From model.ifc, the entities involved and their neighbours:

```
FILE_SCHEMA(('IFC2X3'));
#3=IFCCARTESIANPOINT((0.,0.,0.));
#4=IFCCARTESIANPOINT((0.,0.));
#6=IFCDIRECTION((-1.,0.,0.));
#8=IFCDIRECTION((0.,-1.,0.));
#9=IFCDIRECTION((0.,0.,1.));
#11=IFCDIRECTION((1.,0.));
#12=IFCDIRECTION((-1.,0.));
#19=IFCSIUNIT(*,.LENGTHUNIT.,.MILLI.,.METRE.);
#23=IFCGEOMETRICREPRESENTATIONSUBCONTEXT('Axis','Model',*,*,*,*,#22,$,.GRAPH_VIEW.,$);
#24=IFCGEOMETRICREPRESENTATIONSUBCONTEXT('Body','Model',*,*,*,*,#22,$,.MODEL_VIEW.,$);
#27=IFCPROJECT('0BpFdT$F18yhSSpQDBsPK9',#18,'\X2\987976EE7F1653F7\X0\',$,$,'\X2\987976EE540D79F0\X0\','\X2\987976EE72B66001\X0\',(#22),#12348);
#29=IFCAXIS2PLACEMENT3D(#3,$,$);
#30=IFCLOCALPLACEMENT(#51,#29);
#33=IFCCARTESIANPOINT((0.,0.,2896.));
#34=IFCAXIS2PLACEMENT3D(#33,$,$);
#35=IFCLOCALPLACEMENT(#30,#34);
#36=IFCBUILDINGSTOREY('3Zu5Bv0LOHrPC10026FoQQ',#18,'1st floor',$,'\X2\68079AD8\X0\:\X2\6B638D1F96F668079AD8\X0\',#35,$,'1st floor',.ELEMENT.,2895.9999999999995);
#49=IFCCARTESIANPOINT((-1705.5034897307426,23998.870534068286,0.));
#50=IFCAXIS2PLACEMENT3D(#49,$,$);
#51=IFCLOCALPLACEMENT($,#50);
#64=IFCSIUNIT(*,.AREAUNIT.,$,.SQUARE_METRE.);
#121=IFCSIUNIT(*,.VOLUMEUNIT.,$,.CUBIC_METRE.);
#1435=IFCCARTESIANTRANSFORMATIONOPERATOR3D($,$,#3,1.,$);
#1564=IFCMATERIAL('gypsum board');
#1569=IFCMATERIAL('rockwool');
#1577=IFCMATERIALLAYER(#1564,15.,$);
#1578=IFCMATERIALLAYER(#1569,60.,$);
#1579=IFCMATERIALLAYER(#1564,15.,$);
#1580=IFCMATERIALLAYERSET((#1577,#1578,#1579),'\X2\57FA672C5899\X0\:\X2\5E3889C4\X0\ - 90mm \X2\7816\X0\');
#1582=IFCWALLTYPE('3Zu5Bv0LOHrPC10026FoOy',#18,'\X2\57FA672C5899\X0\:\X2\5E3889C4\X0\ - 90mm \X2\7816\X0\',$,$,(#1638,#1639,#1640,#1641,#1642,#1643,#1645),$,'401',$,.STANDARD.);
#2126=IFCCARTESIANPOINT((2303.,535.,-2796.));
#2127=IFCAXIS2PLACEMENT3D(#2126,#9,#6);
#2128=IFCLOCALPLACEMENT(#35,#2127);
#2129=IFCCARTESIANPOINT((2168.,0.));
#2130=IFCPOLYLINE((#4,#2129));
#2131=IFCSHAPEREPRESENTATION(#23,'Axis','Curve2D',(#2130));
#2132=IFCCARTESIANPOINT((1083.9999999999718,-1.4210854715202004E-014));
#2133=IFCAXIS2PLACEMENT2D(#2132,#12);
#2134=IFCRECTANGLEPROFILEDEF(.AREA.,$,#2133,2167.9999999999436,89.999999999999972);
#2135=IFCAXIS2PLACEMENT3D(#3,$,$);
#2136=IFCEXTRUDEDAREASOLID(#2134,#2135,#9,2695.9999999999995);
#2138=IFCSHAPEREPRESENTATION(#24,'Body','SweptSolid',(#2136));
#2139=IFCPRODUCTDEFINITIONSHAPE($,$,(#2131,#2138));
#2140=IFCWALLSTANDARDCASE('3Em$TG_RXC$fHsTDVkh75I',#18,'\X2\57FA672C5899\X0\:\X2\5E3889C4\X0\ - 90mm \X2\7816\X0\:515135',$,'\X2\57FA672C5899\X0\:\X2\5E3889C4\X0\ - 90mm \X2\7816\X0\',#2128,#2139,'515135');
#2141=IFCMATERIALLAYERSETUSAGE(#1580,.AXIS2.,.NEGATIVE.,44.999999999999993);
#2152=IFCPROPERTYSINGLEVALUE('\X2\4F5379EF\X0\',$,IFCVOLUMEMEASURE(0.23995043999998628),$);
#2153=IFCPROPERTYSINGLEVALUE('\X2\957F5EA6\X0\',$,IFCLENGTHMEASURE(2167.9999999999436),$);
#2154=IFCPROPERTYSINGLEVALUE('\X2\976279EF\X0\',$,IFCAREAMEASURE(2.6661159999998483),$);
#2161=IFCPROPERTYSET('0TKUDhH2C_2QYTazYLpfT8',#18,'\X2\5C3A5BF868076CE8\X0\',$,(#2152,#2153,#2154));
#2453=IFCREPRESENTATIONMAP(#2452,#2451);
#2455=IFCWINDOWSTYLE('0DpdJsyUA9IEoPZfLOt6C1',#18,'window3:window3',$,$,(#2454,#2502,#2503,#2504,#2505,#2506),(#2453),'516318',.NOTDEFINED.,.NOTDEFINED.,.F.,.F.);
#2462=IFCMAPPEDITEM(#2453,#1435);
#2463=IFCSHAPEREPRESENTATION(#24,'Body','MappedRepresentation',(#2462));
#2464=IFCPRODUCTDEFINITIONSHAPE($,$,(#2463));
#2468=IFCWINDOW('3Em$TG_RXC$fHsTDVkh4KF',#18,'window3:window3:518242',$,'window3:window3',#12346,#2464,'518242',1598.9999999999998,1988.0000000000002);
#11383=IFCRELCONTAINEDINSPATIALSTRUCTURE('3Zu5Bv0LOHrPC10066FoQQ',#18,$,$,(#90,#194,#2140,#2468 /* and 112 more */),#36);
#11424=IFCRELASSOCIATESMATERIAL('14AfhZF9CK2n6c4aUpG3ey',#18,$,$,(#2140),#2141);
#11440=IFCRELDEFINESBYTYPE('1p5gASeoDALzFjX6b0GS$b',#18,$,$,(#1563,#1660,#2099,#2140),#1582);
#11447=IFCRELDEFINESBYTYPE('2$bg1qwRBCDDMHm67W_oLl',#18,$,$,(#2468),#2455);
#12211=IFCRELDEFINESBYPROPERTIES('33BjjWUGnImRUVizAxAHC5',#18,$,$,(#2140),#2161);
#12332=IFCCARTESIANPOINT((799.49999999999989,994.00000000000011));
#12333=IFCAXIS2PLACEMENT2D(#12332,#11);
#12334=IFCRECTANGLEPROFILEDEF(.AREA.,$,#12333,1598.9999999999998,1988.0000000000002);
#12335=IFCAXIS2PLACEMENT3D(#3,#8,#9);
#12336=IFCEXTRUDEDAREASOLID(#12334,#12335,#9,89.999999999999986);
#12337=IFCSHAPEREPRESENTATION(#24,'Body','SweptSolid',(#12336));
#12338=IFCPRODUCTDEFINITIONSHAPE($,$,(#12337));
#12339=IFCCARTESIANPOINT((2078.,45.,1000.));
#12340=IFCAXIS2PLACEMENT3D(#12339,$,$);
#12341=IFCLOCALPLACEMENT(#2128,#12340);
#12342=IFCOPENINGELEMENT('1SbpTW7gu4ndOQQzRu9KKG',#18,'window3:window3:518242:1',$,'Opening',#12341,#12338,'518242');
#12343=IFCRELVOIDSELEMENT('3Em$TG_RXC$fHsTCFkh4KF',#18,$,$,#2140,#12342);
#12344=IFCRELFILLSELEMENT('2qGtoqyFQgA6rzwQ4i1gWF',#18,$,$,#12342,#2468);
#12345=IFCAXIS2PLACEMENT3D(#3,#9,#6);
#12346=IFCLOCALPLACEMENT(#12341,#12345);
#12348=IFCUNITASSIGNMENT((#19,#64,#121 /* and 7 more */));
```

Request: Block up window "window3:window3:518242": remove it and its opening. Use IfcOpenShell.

```python
import ifcopenshell
import ifcopenshell.api.feature
import ifcopenshell.api.pset
import ifcopenshell.api.root
import ifcopenshell.geom
import ifcopenshell.util.element
import ifcopenshell.util.shape
import ifcopenshell.util.unit

model = ifcopenshell.open("model.ifc")
area_scale = ifcopenshell.util.unit.calculate_unit_scale(model, "AREAUNIT")
volume_scale = ifcopenshell.util.unit.calculate_unit_scale(model, "VOLUMEUNIT")
settings = ifcopenshell.geom.settings()


def volume(element):
    """Net volume in cubic metres, openings subtracted."""
    shape = ifcopenshell.geom.create_shape(settings, element)
    return ifcopenshell.util.shape.get_volume(shape.geometry)


window = model.by_guid("3Em$TG_RXC$fHsTDVkh4KF")
opening = window.FillsVoids[0].RelatingOpeningElement
wall = opening.VoidsElements[0].RelatingBuildingElement
before = volume(wall)

ifcopenshell.api.root.remove_product(model, product=window)
ifcopenshell.api.feature.remove_feature(model, feature=opening)

after = volume(wall)
thickness = 0.09  # wall thickness in metres

# Update the wall's stored quantities.
pset = model.by_id(ifcopenshell.util.element.get_pset(wall, "尺寸标注", should_inherit=False)["id"])
ifcopenshell.api.pset.edit_pset(model, pset=pset, properties={
    "体积": model.create_entity("IfcVolumeMeasure", after / volume_scale),
    "面积": model.create_entity("IfcAreaMeasure", after / thickness / area_scale),
})

print(f"wall volume {before:.3f} -> {after:.3f} m3")

model.write("model_v2.ifc")
```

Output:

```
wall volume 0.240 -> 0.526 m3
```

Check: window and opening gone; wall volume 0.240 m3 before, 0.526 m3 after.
